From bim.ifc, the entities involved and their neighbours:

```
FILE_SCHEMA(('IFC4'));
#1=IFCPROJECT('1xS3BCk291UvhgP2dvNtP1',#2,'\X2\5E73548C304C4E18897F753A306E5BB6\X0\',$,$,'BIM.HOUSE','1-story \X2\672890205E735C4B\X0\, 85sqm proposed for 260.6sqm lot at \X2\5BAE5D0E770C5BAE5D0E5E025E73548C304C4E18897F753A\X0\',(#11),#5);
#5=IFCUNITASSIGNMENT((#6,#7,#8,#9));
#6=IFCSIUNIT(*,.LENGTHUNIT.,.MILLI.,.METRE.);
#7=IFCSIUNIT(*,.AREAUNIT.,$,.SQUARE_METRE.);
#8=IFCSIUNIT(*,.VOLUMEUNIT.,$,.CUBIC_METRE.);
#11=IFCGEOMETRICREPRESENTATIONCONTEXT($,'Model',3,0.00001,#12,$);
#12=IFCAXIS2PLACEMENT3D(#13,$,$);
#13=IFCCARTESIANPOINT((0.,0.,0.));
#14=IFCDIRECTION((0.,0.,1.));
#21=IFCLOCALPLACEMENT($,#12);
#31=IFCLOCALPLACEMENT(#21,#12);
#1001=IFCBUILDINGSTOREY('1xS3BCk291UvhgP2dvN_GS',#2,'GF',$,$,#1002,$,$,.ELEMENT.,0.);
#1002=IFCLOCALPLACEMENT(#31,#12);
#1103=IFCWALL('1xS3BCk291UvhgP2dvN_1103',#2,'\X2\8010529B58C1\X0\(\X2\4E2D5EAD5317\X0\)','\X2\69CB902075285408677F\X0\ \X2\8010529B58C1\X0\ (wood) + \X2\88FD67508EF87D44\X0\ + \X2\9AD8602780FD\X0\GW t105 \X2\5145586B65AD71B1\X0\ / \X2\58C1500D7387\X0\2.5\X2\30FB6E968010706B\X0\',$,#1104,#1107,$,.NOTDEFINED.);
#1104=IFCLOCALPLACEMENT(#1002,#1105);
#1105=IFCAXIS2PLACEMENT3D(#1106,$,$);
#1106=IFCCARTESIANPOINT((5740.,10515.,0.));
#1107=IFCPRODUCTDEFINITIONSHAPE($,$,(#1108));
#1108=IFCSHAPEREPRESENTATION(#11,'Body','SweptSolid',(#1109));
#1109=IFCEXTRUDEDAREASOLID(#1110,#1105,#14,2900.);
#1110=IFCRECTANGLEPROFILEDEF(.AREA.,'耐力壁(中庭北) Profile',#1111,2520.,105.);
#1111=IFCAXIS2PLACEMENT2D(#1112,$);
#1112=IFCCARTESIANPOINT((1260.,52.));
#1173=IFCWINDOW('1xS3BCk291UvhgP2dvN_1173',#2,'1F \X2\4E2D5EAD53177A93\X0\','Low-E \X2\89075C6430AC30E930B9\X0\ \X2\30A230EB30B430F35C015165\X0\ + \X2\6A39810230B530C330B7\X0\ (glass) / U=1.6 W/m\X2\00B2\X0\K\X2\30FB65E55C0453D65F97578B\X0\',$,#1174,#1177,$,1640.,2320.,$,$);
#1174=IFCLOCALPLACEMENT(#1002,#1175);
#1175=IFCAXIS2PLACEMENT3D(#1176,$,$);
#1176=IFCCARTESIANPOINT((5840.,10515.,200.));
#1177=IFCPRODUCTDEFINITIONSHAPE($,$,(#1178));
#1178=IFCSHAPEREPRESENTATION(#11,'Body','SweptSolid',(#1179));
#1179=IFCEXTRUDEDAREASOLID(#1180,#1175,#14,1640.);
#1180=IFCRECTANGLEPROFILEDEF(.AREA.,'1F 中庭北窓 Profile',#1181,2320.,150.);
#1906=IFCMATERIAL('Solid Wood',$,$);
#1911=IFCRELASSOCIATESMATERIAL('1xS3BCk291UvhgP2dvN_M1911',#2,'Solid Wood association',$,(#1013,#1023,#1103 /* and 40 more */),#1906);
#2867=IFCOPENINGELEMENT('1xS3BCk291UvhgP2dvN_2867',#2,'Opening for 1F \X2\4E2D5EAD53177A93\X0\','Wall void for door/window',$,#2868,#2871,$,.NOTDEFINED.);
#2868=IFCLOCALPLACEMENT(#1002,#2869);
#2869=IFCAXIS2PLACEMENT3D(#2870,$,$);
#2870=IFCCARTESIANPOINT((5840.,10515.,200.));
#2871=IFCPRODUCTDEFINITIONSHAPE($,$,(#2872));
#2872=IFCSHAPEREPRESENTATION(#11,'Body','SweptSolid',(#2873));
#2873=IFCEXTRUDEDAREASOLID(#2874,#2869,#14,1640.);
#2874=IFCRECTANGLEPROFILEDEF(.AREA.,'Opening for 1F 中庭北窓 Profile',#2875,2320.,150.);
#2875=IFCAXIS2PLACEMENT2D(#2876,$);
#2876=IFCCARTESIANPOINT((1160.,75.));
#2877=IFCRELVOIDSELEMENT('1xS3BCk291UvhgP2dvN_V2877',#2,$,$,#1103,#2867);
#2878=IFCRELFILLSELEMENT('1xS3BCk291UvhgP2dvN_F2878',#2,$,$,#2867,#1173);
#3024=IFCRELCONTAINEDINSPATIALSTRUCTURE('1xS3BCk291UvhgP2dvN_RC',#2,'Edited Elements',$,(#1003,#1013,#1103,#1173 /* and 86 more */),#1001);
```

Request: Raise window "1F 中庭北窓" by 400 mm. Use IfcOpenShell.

```python
import numpy as np
import ifcopenshell
import ifcopenshell.api.geometry
import ifcopenshell.util.placement
import ifcopenshell.util.unit

model = ifcopenshell.open("bim.ifc")
unit_scale = ifcopenshell.util.unit.calculate_unit_scale(model)

window = model.by_id(1173)
opening = window.FillsVoids[0].RelatingOpeningElement
dz = 400.0

shift = np.array([0.0, 0.0, dz])
# The window is not placed relative to its opening, so move both.
for product in (opening, window):
    matrix = ifcopenshell.util.placement.get_local_placement(product.ObjectPlacement)
    matrix[:3, 3] += shift
    ifcopenshell.api.geometry.edit_object_placement(model, product=product, matrix=matrix, is_si=False)

print(f"moved by {dz * unit_scale:+.3f} m")

model.write("bim_v2.ifc")
```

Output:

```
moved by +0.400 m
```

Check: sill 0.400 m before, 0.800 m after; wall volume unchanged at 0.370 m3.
